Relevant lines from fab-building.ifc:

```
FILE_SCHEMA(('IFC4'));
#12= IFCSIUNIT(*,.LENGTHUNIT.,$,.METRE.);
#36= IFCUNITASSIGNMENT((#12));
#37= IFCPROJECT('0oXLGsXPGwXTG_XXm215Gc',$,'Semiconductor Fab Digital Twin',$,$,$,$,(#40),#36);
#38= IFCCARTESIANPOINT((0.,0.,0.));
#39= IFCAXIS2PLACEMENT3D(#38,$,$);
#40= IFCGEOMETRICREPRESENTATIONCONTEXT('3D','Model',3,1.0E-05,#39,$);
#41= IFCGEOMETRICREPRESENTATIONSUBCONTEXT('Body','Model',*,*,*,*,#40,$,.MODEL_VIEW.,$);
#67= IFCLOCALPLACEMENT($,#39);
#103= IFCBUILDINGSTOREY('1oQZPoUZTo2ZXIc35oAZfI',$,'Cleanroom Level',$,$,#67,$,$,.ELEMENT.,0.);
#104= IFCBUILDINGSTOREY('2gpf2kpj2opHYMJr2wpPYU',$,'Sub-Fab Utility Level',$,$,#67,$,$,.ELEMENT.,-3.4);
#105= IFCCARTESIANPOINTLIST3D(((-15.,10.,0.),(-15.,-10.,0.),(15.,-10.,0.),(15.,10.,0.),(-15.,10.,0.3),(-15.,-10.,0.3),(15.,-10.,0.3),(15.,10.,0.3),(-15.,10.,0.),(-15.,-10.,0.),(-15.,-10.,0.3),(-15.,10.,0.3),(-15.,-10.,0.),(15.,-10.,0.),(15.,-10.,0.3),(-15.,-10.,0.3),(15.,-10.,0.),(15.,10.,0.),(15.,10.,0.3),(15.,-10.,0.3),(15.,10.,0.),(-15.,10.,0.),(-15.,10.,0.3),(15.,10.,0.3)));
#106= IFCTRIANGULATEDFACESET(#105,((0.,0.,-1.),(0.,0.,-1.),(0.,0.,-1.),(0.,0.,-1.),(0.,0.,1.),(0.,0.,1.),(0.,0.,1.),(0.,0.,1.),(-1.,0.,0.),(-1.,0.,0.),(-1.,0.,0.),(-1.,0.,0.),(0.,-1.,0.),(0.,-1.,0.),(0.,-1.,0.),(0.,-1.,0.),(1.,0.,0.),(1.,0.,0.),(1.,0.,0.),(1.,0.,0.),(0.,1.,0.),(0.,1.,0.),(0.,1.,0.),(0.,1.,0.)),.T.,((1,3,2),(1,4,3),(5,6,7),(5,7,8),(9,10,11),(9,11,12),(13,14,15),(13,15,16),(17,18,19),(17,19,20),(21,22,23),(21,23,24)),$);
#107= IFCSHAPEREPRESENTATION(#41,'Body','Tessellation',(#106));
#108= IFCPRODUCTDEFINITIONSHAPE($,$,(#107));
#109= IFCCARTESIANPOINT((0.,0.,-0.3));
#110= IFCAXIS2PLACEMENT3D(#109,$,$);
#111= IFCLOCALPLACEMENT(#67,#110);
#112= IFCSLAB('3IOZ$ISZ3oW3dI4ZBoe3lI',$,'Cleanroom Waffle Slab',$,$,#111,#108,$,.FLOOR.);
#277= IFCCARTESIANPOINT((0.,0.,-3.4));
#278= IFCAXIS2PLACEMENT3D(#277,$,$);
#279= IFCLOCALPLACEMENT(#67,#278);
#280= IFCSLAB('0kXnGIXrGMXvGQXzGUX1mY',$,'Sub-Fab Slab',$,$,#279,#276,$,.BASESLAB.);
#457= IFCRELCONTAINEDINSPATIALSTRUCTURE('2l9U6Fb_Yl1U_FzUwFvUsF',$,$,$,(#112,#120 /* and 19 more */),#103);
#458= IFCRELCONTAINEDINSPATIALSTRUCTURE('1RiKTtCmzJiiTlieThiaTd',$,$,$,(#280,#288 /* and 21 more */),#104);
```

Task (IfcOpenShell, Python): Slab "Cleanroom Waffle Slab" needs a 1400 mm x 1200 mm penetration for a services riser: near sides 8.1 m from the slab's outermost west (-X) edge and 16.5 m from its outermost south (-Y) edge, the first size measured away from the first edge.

```python
import numpy as np
import ifcopenshell
import ifcopenshell.api.feature
import ifcopenshell.api.geometry
import ifcopenshell.api.root
import ifcopenshell.geom
import ifcopenshell.util.placement
import ifcopenshell.util.representation
import ifcopenshell.util.shape
import ifcopenshell.util.unit

model = ifcopenshell.open("fab-building.ifc")
unit_scale = ifcopenshell.util.unit.calculate_unit_scale(model)
settings = ifcopenshell.geom.settings()


def volume(element):
    """Net volume in cubic metres, openings subtracted."""
    shape = ifcopenshell.geom.create_shape(settings, element)
    return ifcopenshell.util.shape.get_volume(shape.geometry)


slab = model.by_id(112)
before = volume(slab)

# Extent in the slab's own axes, in metres. The edges named are its -X and -Y sides.
slab_shape = ifcopenshell.geom.create_shape(settings, slab)
vertices = ifcopenshell.util.shape.get_vertices(slab_shape.geometry)
x_min, y_min, bottom = vertices.min(axis=0)
top = vertices[:, 2].max()

opening = ifcopenshell.api.root.create_entity(model, ifc_class="IfcOpeningElement", name="Services riser opening", predefined_type="OPENING")
context = ifcopenshell.util.representation.get_context(model, "Model", "Body", "MODEL_VIEW")
width, depth = 1.4, 1.2
outline = [(0.0, 0.0), (width, 0.0), (width, depth), (0.0, depth), (0.0, 0.0)]
# Overshoot both faces by 50 mm so the cut is clean.
shape = ifcopenshell.api.geometry.add_slab_representation(
    model, context=context, depth=top - bottom + 0.1, polyline=outline
)
ifcopenshell.api.geometry.assign_representation(model, product=opening, representation=shape)

matrix = ifcopenshell.util.placement.get_local_placement(slab.ObjectPlacement)
matrix[:, 3] = matrix @ np.append(np.array([x_min + 8.1, y_min + 16.5, bottom - 0.05]) / unit_scale, 1.0)
ifcopenshell.api.geometry.edit_object_placement(model, product=opening, matrix=matrix, is_si=False)
ifcopenshell.api.feature.add_feature(model, feature=opening, element=slab)

after = volume(slab)

print(f"slab volume {before:.3f} -> {after:.3f} m3")

model.write("fab-building-out.ifc")
```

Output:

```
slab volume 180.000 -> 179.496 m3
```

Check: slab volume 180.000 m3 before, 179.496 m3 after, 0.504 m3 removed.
